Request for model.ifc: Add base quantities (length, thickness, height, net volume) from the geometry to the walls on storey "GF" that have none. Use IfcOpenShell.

First a look at what the model holds.

```python
import ifcopenshell
import ifcopenshell.util.element
import ifcopenshell.util.unit

model = ifcopenshell.open("model.ifc")
print(model.schema)
for unit_type in ("LENGTHUNIT", "AREAUNIT", "VOLUMEUNIT"):
    print(unit_type, ifcopenshell.util.unit.calculate_unit_scale(model, unit_type))
storey = next(s for s in model.by_type("IfcBuildingStorey") if s.Name == "GF")
walls = [e for e in ifcopenshell.util.element.get_decomposition(storey) if e.is_a("IfcWall")]
for e in sorted(walls, key=lambda e: e.id()):
    print(e.id(), e.is_a(), e.Name, list(ifcopenshell.util.element.get_psets(e, qtos_only=True)), sep=" | ")
```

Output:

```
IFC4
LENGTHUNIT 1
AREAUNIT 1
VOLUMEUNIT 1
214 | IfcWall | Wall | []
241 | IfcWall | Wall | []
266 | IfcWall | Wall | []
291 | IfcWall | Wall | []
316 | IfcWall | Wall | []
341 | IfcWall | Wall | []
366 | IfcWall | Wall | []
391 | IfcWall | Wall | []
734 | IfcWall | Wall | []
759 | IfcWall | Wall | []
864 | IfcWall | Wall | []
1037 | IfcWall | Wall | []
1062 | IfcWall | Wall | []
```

```python
import ifcopenshell
import ifcopenshell.api.pset
import ifcopenshell.geom
import ifcopenshell.util.element
import ifcopenshell.util.shape
import ifcopenshell.util.unit

model = ifcopenshell.open("model.ifc")
unit_scale = ifcopenshell.util.unit.calculate_unit_scale(model)
volume_scale = ifcopenshell.util.unit.calculate_unit_scale(model, "VOLUMEUNIT")
settings = ifcopenshell.geom.settings()

storey = next(s for s in model.by_type("IfcBuildingStorey") if s.Name == "GF")
walls = [e for e in ifcopenshell.util.element.get_decomposition(storey) if e.is_a("IfcWall")]

for e in sorted(walls, key=lambda e: e.id()):
    if ifcopenshell.util.element.get_psets(e, qtos_only=True, should_inherit=False):
        continue
    # Geometry comes back in metres, in the element's own axes.
    shape = ifcopenshell.geom.create_shape(settings, e)
    values = {
        "Length": ifcopenshell.util.shape.get_x(shape.geometry) / unit_scale,
        "Width": ifcopenshell.util.shape.get_y(shape.geometry) / unit_scale,
        "Height": ifcopenshell.util.shape.get_z(shape.geometry) / unit_scale,
        "NetVolume": ifcopenshell.util.shape.get_volume(shape.geometry) / volume_scale,
    }
    qto = ifcopenshell.api.pset.add_qto(model, product=e, name="Qto_WallBaseQuantities")
    ifcopenshell.api.pset.edit_qto(model, qto=qto, properties=values)
    print(e.id(), {k: round(v, 3) for k, v in values.items()})

model.write("model_edited.ifc")
```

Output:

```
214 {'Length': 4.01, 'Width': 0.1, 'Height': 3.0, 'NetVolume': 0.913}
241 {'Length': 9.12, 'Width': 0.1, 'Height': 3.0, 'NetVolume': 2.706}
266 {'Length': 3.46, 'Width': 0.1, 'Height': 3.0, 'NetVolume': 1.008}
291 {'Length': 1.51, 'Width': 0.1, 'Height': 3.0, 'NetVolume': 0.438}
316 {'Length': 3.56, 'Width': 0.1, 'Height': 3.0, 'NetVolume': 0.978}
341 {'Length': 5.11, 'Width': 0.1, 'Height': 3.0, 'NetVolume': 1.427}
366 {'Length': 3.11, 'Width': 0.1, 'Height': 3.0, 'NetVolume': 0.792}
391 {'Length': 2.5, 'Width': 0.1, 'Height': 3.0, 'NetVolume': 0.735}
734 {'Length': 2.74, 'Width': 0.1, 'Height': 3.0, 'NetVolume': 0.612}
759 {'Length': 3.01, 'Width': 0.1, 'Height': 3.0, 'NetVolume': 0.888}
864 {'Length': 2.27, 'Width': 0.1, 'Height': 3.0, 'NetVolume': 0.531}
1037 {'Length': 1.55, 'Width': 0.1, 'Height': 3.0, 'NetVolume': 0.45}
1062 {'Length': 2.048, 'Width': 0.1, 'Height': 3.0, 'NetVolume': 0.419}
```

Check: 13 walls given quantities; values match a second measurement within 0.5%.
